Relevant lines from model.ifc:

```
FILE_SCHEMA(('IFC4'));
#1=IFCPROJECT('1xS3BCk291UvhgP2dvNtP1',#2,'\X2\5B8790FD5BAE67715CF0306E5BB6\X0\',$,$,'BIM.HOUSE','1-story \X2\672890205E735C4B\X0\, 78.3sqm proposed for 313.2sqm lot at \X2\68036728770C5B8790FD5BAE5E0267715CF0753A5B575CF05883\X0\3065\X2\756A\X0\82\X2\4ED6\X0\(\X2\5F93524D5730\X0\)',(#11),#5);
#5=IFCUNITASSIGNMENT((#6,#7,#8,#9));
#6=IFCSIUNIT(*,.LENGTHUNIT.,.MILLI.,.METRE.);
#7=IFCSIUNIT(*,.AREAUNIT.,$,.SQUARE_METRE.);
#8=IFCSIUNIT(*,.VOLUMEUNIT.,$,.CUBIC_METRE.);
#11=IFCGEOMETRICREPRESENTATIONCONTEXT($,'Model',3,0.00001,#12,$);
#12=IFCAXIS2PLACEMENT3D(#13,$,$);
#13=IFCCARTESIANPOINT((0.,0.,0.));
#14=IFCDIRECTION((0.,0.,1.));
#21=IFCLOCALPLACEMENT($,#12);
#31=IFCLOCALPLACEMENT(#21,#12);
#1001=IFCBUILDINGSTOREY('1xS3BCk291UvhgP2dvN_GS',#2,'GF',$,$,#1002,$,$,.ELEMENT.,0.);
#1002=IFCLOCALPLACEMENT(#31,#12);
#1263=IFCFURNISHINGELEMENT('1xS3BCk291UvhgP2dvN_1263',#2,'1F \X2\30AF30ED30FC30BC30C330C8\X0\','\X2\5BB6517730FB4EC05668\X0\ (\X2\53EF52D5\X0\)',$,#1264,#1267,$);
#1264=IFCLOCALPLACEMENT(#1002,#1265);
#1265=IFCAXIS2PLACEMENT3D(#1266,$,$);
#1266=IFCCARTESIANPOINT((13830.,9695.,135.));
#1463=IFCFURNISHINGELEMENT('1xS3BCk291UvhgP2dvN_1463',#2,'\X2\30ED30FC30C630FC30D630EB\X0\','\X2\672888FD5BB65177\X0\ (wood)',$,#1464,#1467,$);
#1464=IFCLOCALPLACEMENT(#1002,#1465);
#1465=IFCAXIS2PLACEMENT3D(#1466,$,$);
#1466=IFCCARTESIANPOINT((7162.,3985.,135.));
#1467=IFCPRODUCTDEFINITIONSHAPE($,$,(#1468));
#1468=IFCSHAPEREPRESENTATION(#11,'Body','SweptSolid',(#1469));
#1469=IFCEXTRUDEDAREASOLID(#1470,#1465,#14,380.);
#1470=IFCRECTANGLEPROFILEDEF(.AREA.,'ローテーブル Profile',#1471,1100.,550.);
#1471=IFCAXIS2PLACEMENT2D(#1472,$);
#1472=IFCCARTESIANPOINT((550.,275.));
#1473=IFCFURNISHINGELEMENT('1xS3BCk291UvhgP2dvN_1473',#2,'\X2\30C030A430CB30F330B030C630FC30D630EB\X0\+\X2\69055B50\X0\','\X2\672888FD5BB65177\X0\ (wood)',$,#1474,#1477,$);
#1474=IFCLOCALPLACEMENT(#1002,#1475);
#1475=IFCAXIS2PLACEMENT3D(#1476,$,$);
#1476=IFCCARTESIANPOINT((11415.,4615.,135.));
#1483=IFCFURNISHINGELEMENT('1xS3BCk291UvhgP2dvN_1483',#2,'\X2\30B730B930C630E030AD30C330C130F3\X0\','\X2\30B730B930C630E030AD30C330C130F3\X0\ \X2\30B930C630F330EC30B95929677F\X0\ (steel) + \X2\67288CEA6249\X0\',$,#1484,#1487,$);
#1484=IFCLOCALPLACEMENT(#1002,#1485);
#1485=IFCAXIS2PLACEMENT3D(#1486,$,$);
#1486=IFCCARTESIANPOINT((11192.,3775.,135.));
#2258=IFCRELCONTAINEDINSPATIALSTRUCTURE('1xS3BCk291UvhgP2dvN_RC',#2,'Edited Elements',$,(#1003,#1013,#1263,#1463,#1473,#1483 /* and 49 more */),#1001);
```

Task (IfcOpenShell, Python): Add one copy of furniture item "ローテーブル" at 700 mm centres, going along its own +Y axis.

```python
import ifcopenshell
import ifcopenshell.api.geometry
import ifcopenshell.api.root
import ifcopenshell.util.element
import ifcopenshell.util.placement
import ifcopenshell.util.unit

model = ifcopenshell.open("model.ifc")
unit_scale = ifcopenshell.util.unit.calculate_unit_scale(model)


def reuse_history(source, copy):
    """copy_class also copies each property set's owner history, people and application; keep the originals."""
    for rel in copy.IsDefinedBy:
        if rel.is_a("IfcRelDefinesByProperties") and (history := rel.RelatingPropertyDefinition.OwnerHistory):
            rel.RelatingPropertyDefinition.OwnerHistory = source.OwnerHistory
            ifcopenshell.util.element.remove_deep2(model, history)


source = model.by_guid("1xS3BCk291UvhgP2dvN_1463")
base = ifcopenshell.util.placement.get_local_placement(source.ObjectPlacement)
step = base[:3, 1] * 0.7 / unit_scale

for i in range(1, 2):
    copy = ifcopenshell.api.root.copy_class(model, product=source)
    copy.Representation = ifcopenshell.util.element.copy_deep(
        model, source.Representation, exclude=["IfcGeometricRepresentationContext", "IfcRepresentationMap"]
    )
    reuse_history(source, copy)
    matrix = base.copy()
    matrix[:3, 3] += i * step
    print("added at", matrix[:3, 3].round(3) + 0.0)
    ifcopenshell.api.geometry.edit_object_placement(model, product=copy, matrix=matrix, is_si=False)

model.write("model-out.ifc")
```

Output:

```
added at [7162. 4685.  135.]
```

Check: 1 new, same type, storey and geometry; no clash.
